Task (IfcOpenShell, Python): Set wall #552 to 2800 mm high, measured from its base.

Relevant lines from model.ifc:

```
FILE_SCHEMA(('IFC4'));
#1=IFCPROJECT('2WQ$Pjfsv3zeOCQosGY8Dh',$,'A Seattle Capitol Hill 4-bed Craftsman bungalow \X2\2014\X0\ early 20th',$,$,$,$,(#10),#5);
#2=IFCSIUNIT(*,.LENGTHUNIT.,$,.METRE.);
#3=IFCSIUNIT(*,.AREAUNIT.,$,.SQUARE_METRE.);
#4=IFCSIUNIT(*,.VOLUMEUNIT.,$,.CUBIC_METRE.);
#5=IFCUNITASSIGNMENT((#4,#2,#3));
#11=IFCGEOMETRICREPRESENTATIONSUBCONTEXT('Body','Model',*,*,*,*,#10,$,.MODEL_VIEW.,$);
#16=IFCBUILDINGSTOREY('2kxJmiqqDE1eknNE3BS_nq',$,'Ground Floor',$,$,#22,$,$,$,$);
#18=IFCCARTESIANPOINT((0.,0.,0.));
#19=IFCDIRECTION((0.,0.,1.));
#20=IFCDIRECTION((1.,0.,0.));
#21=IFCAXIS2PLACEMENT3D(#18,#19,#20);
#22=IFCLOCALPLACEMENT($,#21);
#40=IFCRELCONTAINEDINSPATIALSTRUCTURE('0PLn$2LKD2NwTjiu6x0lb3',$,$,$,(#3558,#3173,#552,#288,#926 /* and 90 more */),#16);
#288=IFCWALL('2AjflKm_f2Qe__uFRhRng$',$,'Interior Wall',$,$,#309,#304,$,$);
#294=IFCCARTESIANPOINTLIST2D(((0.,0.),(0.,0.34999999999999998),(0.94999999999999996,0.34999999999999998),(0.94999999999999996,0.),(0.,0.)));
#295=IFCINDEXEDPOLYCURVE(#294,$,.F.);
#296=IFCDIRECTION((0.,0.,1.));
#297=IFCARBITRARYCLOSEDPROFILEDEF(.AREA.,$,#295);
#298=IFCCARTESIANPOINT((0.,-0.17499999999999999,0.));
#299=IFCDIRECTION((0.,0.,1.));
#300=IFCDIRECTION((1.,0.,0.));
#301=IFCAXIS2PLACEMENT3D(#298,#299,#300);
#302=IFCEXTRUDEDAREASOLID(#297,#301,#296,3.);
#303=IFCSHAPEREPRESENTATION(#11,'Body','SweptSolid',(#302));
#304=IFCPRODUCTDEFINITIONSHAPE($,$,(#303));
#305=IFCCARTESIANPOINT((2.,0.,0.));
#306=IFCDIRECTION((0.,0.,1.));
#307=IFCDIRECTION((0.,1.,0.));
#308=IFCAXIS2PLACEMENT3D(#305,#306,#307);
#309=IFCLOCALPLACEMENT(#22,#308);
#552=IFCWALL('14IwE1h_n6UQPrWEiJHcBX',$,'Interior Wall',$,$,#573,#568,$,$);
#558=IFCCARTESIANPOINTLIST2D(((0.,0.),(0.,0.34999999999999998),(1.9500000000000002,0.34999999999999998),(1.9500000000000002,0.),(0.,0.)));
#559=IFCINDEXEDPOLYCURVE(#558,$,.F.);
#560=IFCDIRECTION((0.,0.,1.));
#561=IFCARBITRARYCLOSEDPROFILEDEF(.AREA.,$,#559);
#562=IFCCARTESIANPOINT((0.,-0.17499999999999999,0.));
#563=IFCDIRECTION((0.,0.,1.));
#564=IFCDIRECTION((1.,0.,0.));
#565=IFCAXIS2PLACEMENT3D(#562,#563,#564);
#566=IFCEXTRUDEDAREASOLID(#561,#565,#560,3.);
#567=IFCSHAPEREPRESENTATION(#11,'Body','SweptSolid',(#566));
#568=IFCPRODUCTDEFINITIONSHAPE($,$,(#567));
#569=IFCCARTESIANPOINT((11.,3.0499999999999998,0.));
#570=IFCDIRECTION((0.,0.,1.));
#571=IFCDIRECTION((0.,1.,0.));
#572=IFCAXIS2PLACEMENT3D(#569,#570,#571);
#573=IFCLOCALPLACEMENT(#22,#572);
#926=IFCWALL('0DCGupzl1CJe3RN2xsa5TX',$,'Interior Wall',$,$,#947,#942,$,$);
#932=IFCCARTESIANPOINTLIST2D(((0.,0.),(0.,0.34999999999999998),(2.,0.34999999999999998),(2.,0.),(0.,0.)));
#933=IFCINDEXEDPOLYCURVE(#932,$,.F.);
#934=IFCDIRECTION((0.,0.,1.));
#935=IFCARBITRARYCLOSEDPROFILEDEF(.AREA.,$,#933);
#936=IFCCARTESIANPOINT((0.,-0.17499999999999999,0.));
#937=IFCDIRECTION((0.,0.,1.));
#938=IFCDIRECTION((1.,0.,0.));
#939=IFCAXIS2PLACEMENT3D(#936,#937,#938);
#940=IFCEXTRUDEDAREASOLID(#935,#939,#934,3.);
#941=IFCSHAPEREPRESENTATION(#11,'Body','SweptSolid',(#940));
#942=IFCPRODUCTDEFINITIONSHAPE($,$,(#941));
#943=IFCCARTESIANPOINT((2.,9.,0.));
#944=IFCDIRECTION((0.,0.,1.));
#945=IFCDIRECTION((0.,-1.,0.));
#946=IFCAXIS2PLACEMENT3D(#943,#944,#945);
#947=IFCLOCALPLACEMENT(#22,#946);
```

```python
import ifcopenshell
import ifcopenshell.geom
import ifcopenshell.util.representation
import ifcopenshell.util.shape

model = ifcopenshell.open("model.ifc")
settings = ifcopenshell.geom.settings()


def volume(element):
    """Net volume in cubic metres, openings subtracted."""
    shape = ifcopenshell.geom.create_shape(settings, element)
    return ifcopenshell.util.shape.get_volume(shape.geometry)


wall = model.by_guid("14IwE1h_n6UQPrWEiJHcBX")
before = volume(wall)

body = ifcopenshell.util.representation.get_representation(wall, "Model", "Body")
solid = body.Items[0]
old_height = solid.Depth
solid.Depth = 2.8
after = volume(wall)

print(f"height {old_height:g} -> {solid.Depth:g}, volume {before:.3f} -> {after:.3f} m3")

model.write("model_updated.ifc")
```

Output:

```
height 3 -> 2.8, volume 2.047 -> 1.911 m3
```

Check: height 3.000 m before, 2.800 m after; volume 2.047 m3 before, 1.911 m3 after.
